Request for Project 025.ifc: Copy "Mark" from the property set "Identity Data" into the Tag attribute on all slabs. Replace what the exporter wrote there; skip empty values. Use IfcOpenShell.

First a look at what the model holds.

```python
import ifcopenshell
import ifcopenshell.util.element

model = ifcopenshell.open("Project 025.ifc")
print(model.schema)
slabs = model.by_type("IfcSlab")
print(len(slabs), "slabs")
for e in slabs[:8]:
    source = ifcopenshell.util.element.get_pset(e, "Identity Data", "Mark")
    target = e.Tag
    print(e.id(), repr(source), repr(target), sep=" | ")
```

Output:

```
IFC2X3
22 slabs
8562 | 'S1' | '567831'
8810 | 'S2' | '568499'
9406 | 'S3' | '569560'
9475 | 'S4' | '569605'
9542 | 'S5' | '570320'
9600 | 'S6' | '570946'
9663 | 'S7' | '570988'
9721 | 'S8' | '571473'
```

```python
import ifcopenshell
import ifcopenshell.util.element

model = ifcopenshell.open("Project 025.ifc")

count = 0
for e in model.by_type("IfcSlab"):
    value = ifcopenshell.util.element.get_pset(e, "Identity Data", "Mark")
    current = e.Tag
    if not value or not value.strip() or current == value:
        continue
    e.Tag = value
    count += 1

print(count, "slabs updated")

model.write("Project 025-out.ifc")
```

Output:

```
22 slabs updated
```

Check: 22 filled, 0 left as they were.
